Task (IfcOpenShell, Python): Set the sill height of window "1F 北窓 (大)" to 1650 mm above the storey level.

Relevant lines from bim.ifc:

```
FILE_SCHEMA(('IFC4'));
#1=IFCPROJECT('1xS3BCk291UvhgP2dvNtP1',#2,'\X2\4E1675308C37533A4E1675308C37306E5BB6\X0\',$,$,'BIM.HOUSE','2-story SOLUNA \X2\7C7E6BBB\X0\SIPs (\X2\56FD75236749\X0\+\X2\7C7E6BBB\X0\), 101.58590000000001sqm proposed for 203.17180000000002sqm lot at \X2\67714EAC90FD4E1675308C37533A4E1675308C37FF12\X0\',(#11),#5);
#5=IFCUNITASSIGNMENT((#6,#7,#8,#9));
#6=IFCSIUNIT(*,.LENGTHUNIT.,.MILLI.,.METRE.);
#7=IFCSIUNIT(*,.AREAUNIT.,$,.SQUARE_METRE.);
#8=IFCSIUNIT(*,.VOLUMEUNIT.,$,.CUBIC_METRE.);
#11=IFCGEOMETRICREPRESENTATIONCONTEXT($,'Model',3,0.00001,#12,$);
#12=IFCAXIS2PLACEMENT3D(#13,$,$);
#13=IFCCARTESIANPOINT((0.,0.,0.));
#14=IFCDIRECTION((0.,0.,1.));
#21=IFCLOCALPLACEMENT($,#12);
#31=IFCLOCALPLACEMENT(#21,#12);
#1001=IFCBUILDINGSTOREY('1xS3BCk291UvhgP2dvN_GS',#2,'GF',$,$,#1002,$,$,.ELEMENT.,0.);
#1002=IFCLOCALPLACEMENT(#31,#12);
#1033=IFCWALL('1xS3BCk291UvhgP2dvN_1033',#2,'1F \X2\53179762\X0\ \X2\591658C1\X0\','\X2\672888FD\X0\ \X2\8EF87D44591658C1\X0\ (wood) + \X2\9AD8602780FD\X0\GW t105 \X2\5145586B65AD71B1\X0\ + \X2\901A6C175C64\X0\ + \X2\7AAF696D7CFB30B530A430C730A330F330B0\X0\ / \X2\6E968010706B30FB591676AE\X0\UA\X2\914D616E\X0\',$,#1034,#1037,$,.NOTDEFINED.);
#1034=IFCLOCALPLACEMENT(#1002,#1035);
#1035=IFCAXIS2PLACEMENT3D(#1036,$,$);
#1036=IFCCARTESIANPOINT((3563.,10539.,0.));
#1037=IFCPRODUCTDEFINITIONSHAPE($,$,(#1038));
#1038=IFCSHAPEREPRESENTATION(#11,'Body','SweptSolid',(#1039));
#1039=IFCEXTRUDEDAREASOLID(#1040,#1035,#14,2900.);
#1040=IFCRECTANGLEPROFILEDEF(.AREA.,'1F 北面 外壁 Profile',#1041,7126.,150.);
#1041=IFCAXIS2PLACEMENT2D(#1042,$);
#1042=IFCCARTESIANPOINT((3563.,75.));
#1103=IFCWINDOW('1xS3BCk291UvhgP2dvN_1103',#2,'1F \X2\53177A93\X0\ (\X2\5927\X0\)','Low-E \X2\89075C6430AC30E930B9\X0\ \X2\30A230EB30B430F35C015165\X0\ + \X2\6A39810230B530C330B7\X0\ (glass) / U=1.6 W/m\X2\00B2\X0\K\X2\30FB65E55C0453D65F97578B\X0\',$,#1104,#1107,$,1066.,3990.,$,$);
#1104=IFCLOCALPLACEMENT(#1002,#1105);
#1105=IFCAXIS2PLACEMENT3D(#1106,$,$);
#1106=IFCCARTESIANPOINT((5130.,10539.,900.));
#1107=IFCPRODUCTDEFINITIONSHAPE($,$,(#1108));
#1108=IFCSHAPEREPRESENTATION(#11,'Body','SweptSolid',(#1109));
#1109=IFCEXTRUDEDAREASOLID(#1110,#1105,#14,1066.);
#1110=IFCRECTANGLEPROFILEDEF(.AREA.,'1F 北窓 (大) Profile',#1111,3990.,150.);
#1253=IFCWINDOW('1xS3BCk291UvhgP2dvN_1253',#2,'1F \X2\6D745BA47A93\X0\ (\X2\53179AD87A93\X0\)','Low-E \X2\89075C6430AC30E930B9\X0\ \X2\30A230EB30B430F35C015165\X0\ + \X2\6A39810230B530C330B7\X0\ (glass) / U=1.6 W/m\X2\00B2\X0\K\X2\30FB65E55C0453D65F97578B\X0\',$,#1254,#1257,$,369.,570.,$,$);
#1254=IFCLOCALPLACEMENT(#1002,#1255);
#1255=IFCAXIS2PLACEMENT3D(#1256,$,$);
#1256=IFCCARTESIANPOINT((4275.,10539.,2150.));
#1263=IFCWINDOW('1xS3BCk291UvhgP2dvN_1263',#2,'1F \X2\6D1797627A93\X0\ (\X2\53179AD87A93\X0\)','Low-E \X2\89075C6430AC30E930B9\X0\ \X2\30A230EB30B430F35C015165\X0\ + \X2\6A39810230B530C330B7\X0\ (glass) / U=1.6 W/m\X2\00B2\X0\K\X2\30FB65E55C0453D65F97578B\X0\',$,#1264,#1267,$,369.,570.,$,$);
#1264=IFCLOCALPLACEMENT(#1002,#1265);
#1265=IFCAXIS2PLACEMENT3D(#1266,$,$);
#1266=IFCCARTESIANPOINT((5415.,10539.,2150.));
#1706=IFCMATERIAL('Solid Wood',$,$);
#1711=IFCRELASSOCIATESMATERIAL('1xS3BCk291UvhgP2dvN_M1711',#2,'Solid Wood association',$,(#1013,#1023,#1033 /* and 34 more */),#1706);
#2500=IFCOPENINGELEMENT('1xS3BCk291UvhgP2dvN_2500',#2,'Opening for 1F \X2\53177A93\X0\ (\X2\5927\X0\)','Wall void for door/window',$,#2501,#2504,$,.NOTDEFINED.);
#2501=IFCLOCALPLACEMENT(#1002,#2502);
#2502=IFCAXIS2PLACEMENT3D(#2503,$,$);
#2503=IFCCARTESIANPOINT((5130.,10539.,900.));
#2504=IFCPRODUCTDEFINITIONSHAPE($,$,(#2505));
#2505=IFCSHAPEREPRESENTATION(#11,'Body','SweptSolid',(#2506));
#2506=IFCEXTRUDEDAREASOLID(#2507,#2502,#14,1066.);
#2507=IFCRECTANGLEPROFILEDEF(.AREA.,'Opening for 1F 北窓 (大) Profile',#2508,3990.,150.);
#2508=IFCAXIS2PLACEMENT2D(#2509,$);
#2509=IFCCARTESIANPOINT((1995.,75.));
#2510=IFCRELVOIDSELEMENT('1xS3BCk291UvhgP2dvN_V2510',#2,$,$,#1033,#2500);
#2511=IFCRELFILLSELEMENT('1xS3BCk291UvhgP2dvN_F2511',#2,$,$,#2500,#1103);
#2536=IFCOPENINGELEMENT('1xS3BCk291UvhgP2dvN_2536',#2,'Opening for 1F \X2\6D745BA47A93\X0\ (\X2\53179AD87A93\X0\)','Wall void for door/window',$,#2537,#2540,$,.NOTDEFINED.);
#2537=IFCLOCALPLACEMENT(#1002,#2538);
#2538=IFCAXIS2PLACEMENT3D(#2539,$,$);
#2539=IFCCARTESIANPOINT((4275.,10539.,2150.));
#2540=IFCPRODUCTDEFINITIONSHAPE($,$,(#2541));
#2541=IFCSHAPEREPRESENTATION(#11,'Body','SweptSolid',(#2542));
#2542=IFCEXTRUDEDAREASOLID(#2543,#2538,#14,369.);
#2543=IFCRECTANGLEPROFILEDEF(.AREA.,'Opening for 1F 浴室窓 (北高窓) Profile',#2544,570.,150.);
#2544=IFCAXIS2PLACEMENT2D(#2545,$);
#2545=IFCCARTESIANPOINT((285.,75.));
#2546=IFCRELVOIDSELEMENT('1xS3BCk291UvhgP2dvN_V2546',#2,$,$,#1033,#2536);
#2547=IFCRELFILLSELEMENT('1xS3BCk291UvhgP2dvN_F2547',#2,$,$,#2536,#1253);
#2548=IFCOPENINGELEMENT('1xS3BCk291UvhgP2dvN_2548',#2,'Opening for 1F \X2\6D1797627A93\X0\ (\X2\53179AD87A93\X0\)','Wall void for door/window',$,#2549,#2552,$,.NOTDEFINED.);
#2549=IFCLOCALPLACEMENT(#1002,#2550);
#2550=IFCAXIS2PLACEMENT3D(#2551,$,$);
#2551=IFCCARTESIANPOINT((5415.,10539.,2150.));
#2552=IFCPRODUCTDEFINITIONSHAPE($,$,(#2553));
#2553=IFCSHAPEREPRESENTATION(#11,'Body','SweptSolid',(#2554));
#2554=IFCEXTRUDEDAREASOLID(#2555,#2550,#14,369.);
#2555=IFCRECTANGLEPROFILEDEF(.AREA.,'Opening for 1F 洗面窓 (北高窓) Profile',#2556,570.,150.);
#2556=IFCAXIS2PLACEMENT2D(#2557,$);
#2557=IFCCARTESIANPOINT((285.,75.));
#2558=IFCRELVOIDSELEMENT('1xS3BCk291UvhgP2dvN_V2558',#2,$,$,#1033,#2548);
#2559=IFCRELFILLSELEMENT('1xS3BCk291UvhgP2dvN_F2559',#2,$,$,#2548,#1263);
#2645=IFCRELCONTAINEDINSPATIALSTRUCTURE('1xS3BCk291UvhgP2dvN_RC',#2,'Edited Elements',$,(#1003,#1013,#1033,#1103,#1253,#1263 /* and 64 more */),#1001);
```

```python
import numpy as np
import ifcopenshell
import ifcopenshell.api.geometry
import ifcopenshell.geom
import ifcopenshell.util.element
import ifcopenshell.util.placement
import ifcopenshell.util.shape
import ifcopenshell.util.unit

model = ifcopenshell.open("bim.ifc")
unit_scale = ifcopenshell.util.unit.calculate_unit_scale(model)

window = model.by_guid("1xS3BCk291UvhgP2dvN_1103")
opening = window.FillsVoids[0].RelatingOpeningElement
storey = ifcopenshell.util.element.get_container(window, ifc_class="IfcBuildingStorey")
level = ifcopenshell.util.placement.get_local_placement(storey.ObjectPlacement)[2, 3]

# The opening's origin need not be at the sill, so measure its lowest point.
shape = ifcopenshell.geom.create_shape(ifcopenshell.geom.settings(), opening)
bottom = ifcopenshell.util.shape.get_shape_bottom_elevation(shape, shape.geometry) / unit_scale
dz = level + 1650.0 - bottom

shift = np.array([0.0, 0.0, dz])
# The window is not placed relative to its opening, so move both.
for product in (opening, window):
    matrix = ifcopenshell.util.placement.get_local_placement(product.ObjectPlacement)
    matrix[:3, 3] += shift
    ifcopenshell.api.geometry.edit_object_placement(model, product=product, matrix=matrix, is_si=False)

print(f"moved by {dz * unit_scale:+.3f} m")

model.write("bim_updated.ifc")
```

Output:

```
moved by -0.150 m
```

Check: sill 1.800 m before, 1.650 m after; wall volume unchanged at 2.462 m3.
